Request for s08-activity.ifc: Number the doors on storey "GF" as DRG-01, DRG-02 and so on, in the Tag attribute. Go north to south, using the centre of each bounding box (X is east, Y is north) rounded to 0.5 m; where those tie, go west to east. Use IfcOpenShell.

First a look at what the model holds.

```python
import ifcopenshell
import ifcopenshell.util.element
import ifcopenshell.util.placement

model = ifcopenshell.open("s08-activity.ifc")
print(model.schema)
storey = next(s for s in model.by_type("IfcBuildingStorey") if s.Name == "GF")
doors = [e for e in ifcopenshell.util.element.get_decomposition(storey) if e.is_a("IfcDoor")]
for e in sorted(doors, key=lambda e: e.id()):
    origin = ifcopenshell.util.placement.get_local_placement(e.ObjectPlacement)[:3, 3]
    print(e.id(), e.Tag, e.Name, origin.round(2) + 0.0, sep=" | ")
```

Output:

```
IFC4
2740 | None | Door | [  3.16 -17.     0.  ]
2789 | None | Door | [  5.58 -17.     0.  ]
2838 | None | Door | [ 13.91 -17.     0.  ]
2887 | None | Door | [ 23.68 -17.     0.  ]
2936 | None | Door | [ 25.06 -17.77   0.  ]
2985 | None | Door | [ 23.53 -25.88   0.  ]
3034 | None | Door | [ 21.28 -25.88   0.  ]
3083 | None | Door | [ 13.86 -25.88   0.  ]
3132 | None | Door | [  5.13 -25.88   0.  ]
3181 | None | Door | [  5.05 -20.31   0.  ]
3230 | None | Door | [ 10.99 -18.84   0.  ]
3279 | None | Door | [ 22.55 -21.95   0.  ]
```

```python
import ifcopenshell
import ifcopenshell.geom
import ifcopenshell.util.element
import ifcopenshell.util.shape

model = ifcopenshell.open("s08-activity.ifc")
settings = ifcopenshell.geom.settings()
settings.set("use-world-coords", True)


def centre(element):
    shape = ifcopenshell.geom.create_shape(settings, element)
    return ifcopenshell.util.shape.get_bbox_centroid(shape.geometry)


storey = next(s for s in model.by_type("IfcBuildingStorey") if s.Name == "GF")
doors = [e for e in ifcopenshell.util.element.get_decomposition(storey) if e.is_a("IfcDoor")]

# Insertion points can sit at a corner or the storey origin, so sort by the geometry (in metres).
centres = {e: centre(e) for e in doors}
doors.sort(key=lambda e: (-round(centres[e][1] / 0.5), centres[e][0]))

for i, e in enumerate(doors, start=1):
    number = f"DRG-{i:02d}"
    e.Tag = number
    print(e.id(), number)

model.write("s08-activity_rev.ifc")
```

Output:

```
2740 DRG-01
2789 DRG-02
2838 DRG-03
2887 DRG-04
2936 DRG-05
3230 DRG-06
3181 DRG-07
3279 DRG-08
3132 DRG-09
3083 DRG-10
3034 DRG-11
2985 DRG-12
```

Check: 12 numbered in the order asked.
